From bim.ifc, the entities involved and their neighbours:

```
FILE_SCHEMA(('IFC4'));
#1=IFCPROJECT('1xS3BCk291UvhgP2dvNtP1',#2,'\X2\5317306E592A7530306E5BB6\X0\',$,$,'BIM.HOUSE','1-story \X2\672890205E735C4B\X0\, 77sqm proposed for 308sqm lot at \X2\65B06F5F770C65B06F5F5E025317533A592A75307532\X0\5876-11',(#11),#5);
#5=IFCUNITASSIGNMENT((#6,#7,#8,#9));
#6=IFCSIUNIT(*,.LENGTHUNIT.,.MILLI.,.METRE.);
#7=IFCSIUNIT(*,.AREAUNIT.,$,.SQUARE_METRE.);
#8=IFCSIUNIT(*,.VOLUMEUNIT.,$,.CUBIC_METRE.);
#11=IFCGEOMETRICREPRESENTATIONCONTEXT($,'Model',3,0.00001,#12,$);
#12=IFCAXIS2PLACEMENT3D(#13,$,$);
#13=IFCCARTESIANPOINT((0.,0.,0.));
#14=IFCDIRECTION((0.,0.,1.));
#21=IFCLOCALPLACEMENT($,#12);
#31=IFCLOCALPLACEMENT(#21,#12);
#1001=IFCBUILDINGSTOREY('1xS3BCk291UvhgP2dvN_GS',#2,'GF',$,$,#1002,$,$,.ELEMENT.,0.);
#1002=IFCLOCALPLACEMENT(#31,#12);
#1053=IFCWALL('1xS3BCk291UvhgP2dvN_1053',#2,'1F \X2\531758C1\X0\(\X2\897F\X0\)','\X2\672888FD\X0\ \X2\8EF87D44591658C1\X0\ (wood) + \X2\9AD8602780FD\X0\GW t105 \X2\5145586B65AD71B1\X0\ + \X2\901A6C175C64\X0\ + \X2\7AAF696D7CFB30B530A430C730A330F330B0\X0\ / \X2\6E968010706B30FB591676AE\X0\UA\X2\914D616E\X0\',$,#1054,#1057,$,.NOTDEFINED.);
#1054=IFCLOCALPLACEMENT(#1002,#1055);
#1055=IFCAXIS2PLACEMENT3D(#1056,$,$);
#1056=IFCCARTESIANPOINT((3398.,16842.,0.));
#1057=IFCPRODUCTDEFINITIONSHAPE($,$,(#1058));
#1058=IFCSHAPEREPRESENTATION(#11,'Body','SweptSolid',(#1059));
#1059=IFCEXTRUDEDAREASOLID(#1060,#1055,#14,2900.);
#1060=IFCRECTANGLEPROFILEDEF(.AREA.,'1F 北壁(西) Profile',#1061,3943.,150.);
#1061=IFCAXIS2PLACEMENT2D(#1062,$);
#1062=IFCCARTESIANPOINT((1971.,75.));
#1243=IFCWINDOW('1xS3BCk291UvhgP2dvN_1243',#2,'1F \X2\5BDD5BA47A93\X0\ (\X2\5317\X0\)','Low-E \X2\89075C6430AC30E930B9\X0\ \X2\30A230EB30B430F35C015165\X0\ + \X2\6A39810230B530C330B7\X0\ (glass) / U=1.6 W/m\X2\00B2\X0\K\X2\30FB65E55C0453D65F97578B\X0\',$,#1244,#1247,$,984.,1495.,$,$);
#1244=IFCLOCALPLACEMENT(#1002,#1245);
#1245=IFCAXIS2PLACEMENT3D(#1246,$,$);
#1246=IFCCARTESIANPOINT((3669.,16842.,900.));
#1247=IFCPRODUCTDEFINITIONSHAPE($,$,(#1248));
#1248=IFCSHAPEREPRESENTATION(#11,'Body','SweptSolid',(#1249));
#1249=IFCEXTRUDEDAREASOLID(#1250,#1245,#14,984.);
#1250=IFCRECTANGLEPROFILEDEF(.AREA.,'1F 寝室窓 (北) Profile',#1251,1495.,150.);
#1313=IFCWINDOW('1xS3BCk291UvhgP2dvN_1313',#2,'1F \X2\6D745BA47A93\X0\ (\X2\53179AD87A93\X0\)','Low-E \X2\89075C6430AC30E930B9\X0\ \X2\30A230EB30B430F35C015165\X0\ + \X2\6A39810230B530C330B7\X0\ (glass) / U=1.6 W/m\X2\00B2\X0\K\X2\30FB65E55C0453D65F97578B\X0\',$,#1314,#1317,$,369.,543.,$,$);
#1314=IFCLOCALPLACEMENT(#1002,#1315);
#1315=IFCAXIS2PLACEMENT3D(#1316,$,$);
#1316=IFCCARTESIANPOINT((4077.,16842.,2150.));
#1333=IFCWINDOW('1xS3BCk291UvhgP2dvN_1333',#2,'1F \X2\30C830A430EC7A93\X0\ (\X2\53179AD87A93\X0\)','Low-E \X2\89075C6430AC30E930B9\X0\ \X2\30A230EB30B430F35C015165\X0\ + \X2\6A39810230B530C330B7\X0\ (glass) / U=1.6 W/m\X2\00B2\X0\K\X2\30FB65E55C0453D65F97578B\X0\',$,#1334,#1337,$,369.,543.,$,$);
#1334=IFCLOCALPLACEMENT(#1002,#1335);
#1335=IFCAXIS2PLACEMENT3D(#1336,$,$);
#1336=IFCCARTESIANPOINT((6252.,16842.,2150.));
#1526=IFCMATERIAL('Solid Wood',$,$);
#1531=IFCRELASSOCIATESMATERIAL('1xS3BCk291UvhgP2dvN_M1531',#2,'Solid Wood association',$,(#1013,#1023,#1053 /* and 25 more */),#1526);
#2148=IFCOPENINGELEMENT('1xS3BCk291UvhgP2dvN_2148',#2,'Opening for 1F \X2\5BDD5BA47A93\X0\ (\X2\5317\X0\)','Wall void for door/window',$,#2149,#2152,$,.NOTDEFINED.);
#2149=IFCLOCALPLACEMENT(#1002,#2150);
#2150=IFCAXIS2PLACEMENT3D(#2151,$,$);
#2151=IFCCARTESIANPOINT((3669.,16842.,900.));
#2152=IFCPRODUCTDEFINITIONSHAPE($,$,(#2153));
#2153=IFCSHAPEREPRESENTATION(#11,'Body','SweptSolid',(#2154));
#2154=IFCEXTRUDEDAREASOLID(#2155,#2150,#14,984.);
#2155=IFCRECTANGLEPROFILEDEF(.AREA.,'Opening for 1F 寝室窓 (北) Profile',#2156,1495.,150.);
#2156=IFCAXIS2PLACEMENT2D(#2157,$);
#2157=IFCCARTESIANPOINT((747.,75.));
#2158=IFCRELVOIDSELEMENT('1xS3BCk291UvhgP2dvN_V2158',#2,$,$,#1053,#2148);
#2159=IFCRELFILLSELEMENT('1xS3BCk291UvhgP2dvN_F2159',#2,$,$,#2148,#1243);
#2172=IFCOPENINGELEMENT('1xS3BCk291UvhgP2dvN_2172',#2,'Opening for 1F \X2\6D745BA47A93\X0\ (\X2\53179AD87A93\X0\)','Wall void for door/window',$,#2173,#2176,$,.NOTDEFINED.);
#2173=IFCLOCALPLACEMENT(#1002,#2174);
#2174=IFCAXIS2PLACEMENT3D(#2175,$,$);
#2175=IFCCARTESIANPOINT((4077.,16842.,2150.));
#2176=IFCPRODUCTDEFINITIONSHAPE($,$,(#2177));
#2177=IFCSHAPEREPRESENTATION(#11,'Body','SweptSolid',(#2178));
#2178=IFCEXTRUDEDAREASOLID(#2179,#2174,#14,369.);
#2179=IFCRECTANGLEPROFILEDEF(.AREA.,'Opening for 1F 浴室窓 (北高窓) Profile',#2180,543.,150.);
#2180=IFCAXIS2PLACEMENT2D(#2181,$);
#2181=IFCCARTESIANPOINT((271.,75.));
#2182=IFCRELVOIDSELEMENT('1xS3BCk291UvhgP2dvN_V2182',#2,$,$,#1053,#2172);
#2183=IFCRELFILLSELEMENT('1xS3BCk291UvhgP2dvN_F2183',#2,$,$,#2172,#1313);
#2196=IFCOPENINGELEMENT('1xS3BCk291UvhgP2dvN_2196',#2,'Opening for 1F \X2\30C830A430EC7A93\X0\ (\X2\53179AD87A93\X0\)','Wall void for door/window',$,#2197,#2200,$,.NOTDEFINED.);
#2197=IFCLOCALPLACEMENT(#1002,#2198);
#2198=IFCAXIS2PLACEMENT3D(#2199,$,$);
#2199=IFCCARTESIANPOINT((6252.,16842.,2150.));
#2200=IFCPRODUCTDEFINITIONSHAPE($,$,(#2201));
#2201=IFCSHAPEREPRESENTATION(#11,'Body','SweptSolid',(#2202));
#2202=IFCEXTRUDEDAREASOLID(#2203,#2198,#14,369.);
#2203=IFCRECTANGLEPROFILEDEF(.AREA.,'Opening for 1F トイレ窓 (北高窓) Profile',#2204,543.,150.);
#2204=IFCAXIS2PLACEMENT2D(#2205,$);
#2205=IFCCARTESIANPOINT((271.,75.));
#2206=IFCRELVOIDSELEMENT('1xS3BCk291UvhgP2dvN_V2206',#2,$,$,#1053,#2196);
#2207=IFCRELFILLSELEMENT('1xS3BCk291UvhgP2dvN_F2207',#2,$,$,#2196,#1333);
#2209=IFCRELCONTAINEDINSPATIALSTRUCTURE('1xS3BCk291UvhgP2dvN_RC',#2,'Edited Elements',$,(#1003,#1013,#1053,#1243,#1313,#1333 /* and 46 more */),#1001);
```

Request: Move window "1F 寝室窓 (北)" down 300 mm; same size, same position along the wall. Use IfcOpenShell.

```python
import numpy as np
import ifcopenshell
import ifcopenshell.api.geometry
import ifcopenshell.util.placement
import ifcopenshell.util.unit

model = ifcopenshell.open("bim.ifc")
unit_scale = ifcopenshell.util.unit.calculate_unit_scale(model)

window = model.by_id(1243)
opening = window.FillsVoids[0].RelatingOpeningElement
dz = -0.3 / unit_scale

shift = np.array([0.0, 0.0, dz])
# The window is not placed relative to its opening, so move both.
for product in (opening, window):
    matrix = ifcopenshell.util.placement.get_local_placement(product.ObjectPlacement)
    matrix[:3, 3] += shift
    ifcopenshell.api.geometry.edit_object_placement(model, product=product, matrix=matrix, is_si=False)

print(f"moved by {dz * unit_scale:+.3f} m")

model.write("bim-out.ifc")
```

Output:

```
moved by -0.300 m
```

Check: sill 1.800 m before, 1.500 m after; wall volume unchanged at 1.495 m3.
